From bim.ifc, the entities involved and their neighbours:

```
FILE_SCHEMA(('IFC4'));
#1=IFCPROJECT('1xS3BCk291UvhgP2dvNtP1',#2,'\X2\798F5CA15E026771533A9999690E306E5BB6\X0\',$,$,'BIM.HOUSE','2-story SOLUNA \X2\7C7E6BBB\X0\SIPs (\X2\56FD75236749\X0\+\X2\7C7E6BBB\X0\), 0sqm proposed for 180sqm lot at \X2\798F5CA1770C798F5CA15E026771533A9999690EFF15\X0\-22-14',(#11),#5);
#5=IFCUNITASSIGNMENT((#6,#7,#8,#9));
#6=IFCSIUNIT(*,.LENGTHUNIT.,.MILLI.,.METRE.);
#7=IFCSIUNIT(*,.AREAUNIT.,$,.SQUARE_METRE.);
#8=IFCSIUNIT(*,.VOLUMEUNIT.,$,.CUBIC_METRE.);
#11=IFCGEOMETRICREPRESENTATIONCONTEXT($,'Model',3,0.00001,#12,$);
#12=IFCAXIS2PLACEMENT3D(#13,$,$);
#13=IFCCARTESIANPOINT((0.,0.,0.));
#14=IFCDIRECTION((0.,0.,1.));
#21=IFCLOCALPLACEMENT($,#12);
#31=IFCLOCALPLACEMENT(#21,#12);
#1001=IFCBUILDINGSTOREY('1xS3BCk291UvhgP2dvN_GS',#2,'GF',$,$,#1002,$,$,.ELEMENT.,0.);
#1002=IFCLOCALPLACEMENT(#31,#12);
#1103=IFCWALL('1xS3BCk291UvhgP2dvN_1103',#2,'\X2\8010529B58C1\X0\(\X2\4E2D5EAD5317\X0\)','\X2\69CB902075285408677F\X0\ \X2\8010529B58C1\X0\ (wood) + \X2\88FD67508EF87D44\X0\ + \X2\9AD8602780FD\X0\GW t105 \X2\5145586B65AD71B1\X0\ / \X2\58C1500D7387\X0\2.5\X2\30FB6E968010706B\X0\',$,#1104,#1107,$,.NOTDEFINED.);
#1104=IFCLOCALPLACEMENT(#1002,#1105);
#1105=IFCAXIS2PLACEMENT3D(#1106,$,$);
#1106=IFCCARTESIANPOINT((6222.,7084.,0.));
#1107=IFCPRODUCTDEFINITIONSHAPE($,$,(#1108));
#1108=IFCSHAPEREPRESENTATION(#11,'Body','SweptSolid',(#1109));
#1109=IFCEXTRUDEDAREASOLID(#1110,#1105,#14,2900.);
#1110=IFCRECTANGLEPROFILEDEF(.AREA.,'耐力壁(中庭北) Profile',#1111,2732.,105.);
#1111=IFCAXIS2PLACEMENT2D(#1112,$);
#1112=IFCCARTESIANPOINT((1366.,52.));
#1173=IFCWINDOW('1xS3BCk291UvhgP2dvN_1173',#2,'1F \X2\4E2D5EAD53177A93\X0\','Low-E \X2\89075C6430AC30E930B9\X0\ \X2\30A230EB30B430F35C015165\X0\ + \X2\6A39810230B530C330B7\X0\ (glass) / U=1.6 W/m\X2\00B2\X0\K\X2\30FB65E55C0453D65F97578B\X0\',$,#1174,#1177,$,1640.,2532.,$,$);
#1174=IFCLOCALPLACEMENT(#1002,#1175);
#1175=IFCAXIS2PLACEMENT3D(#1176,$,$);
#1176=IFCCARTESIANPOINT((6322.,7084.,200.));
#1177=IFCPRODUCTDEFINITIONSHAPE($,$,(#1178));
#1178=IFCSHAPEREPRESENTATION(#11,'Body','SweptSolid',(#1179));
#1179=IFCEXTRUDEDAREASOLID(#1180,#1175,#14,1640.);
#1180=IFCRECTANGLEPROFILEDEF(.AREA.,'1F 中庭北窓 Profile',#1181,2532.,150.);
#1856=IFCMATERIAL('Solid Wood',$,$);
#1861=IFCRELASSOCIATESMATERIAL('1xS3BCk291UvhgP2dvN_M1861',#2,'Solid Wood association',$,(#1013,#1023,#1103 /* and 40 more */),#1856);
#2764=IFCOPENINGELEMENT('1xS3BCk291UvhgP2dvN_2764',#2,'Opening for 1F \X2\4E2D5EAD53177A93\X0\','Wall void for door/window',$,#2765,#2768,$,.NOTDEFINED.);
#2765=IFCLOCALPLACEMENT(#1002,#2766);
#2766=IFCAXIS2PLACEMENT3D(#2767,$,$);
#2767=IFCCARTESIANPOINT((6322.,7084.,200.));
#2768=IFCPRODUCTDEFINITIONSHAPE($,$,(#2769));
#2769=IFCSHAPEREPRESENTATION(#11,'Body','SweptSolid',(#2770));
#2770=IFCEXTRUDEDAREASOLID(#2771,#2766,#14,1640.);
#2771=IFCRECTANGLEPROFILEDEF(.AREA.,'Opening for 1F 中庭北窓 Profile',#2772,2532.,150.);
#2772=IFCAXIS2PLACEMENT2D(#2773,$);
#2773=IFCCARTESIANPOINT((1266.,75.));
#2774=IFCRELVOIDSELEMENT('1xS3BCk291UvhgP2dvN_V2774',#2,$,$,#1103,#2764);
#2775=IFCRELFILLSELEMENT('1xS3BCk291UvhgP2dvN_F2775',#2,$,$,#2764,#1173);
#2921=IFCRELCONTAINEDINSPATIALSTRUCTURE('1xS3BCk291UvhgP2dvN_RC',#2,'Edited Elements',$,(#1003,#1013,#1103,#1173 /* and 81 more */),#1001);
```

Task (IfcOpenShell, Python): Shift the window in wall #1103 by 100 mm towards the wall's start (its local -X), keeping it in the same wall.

```python
import ifcopenshell
import ifcopenshell.api.geometry
import ifcopenshell.util.placement
import ifcopenshell.util.unit

model = ifcopenshell.open("bim.ifc")
unit_scale = ifcopenshell.util.unit.calculate_unit_scale(model)

window = model.by_id(1173)
opening = window.FillsVoids[0].RelatingOpeningElement
wall = opening.VoidsElements[0].RelatingBuildingElement

wall_matrix = ifcopenshell.util.placement.get_local_placement(wall.ObjectPlacement)
shift = wall_matrix[:3, 0] * -0.1 / unit_scale
before = ifcopenshell.util.placement.get_local_placement(window.ObjectPlacement)[:3, 3].copy()

# The window is not placed relative to its opening, so move both.
for product in (opening, window):
    matrix = ifcopenshell.util.placement.get_local_placement(product.ObjectPlacement)
    matrix[:3, 3] += shift
    ifcopenshell.api.geometry.edit_object_placement(model, product=product, matrix=matrix, is_si=False)

after = ifcopenshell.util.placement.get_local_placement(window.ObjectPlacement)[:3, 3]
print("window moved by", (after - before).round(3) + 0.0)

model.write("bim_updated.ifc")
```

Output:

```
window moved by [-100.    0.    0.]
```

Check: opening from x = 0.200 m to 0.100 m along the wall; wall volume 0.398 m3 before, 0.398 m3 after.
